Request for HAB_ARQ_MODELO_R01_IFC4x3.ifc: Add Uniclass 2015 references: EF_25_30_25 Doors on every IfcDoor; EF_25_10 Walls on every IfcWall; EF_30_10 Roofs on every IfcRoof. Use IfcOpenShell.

First a look at what the model holds.

```python
import ifcopenshell

model = ifcopenshell.open("HAB_ARQ_MODELO_R01_IFC4x3.ifc")
print(model.schema)
print("classifications:", [c.Name for c in model.by_type("IfcClassification")])
for ifc_class in ("IfcDoor", "IfcRoof", "IfcStair", "IfcWall", "IfcWindow"):
    print(ifc_class, len(model.by_type(ifc_class)))
```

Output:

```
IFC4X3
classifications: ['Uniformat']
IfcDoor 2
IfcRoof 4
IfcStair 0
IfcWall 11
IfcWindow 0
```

```python
import ifcopenshell
import ifcopenshell.api.classification

model = ifcopenshell.open("HAB_ARQ_MODELO_R01_IFC4x3.ifc")

system = ifcopenshell.api.classification.add_classification(model, classification="Uniclass 2015")

codes = {
    "IfcDoor": ("EF_25_30_25", "Doors"),
    "IfcWall": ("EF_25_10", "Walls"),
    "IfcRoof": ("EF_30_10", "Roofs"),
}
for ifc_class, (code, name) in codes.items():
    products = model.by_type(ifc_class)
    ifcopenshell.api.classification.add_reference(
        model, products=products, classification=system, identification=code, name=name
    )
    print(code, len(products))

model.write("HAB_ARQ_MODELO_R01_IFC4x3_rev.ifc")
```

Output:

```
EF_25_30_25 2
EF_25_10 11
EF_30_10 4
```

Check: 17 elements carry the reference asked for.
